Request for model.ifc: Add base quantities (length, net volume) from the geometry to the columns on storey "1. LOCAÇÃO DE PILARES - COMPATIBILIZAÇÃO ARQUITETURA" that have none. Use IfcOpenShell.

First a look at what the model holds.

```python
import ifcopenshell
import ifcopenshell.util.element
import ifcopenshell.util.unit

model = ifcopenshell.open("model.ifc")
print(model.schema)
for unit_type in ("LENGTHUNIT", "AREAUNIT", "VOLUMEUNIT"):
    print(unit_type, ifcopenshell.util.unit.calculate_unit_scale(model, unit_type))
storey = next(s for s in model.by_type("IfcBuildingStorey") if s.Name == "1. LOCAÇÃO DE PILARES - COMPATIBILIZAÇÃO ARQUITETURA")
columns = [e for e in ifcopenshell.util.element.get_decomposition(storey) if e.is_a("IfcColumn")]
for e in sorted(columns, key=lambda e: e.id()):
    print(e.id(), e.is_a(), e.Name, list(ifcopenshell.util.element.get_psets(e, qtos_only=True)), sep=" | ")
```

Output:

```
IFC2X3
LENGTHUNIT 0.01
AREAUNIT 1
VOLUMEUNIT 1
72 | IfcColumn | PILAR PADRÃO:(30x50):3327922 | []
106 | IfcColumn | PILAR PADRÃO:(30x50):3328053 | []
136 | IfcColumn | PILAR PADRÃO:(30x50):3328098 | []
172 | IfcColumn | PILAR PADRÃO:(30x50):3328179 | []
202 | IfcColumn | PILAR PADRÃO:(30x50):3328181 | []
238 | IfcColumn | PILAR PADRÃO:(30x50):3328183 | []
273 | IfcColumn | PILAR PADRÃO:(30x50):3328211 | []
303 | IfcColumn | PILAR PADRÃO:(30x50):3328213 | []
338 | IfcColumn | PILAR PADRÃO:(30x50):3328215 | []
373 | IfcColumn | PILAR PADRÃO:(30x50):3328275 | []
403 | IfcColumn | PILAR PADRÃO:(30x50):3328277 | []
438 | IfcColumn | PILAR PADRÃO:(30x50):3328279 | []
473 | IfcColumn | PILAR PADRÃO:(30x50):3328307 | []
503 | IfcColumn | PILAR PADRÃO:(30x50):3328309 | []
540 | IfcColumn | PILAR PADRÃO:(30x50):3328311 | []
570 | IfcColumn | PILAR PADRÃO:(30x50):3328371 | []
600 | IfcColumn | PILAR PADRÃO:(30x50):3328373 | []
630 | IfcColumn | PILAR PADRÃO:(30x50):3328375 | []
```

```python
import ifcopenshell
import ifcopenshell.api.pset
import ifcopenshell.geom
import ifcopenshell.util.element
import ifcopenshell.util.shape
import ifcopenshell.util.unit

model = ifcopenshell.open("model.ifc")
unit_scale = ifcopenshell.util.unit.calculate_unit_scale(model)
volume_scale = ifcopenshell.util.unit.calculate_unit_scale(model, "VOLUMEUNIT")
settings = ifcopenshell.geom.settings()

storey = next(s for s in model.by_type("IfcBuildingStorey") if s.Name == "1. LOCAÇÃO DE PILARES - COMPATIBILIZAÇÃO ARQUITETURA")
columns = [e for e in ifcopenshell.util.element.get_decomposition(storey) if e.is_a("IfcColumn")]

for e in sorted(columns, key=lambda e: e.id()):
    if ifcopenshell.util.element.get_psets(e, qtos_only=True, should_inherit=False):
        continue
    # Geometry comes back in metres, in the element's own axes.
    shape = ifcopenshell.geom.create_shape(settings, e)
    values = {
        "Length": ifcopenshell.util.shape.get_z(shape.geometry) / unit_scale,
        "NetVolume": ifcopenshell.util.shape.get_volume(shape.geometry) / volume_scale,
    }
    qto = ifcopenshell.api.pset.add_qto(model, product=e, name="BaseQuantities")
    ifcopenshell.api.pset.edit_qto(model, qto=qto, properties=values)
    print(e.id(), {k: round(v, 3) for k, v in values.items()})

model.write("model_v2.ifc")
```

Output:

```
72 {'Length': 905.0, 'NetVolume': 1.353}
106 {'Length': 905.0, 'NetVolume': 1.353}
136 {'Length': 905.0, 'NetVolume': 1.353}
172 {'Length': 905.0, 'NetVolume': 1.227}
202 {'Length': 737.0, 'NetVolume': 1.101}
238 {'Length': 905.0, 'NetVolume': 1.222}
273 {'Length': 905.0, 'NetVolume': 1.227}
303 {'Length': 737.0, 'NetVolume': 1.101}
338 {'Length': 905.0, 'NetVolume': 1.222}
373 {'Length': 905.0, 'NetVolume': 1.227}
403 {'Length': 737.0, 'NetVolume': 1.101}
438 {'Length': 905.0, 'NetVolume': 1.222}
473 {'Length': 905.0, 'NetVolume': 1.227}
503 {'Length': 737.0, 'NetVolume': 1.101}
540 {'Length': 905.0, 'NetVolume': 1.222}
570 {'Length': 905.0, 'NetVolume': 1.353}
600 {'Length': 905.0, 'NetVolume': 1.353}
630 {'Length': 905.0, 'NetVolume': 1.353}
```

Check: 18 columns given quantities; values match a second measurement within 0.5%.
